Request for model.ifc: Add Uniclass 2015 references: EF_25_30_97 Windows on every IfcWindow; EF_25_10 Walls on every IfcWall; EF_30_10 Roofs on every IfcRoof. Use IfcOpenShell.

First a look at what the model holds.

```python
import ifcopenshell

model = ifcopenshell.open("model.ifc")
print(model.schema)
print("classifications:", [c.Name for c in model.by_type("IfcClassification")])
for ifc_class in ("IfcDoor", "IfcRoof", "IfcStair", "IfcWall", "IfcWindow"):
    print(ifc_class, len(model.by_type(ifc_class)))
```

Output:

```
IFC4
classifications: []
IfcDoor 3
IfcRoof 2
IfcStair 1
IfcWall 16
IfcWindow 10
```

```python
import ifcopenshell
import ifcopenshell.api.classification

model = ifcopenshell.open("model.ifc")

system = ifcopenshell.api.classification.add_classification(model, classification="Uniclass 2015")

codes = {
    "IfcWindow": ("EF_25_30_97", "Windows"),
    "IfcWall": ("EF_25_10", "Walls"),
    "IfcRoof": ("EF_30_10", "Roofs"),
}
for ifc_class, (code, name) in codes.items():
    products = model.by_type(ifc_class)
    ifcopenshell.api.classification.add_reference(
        model, products=products, classification=system, identification=code, name=name
    )
    print(code, len(products))

model.write("model_rev.ifc")
```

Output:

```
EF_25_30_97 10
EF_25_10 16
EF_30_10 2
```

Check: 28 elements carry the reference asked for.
